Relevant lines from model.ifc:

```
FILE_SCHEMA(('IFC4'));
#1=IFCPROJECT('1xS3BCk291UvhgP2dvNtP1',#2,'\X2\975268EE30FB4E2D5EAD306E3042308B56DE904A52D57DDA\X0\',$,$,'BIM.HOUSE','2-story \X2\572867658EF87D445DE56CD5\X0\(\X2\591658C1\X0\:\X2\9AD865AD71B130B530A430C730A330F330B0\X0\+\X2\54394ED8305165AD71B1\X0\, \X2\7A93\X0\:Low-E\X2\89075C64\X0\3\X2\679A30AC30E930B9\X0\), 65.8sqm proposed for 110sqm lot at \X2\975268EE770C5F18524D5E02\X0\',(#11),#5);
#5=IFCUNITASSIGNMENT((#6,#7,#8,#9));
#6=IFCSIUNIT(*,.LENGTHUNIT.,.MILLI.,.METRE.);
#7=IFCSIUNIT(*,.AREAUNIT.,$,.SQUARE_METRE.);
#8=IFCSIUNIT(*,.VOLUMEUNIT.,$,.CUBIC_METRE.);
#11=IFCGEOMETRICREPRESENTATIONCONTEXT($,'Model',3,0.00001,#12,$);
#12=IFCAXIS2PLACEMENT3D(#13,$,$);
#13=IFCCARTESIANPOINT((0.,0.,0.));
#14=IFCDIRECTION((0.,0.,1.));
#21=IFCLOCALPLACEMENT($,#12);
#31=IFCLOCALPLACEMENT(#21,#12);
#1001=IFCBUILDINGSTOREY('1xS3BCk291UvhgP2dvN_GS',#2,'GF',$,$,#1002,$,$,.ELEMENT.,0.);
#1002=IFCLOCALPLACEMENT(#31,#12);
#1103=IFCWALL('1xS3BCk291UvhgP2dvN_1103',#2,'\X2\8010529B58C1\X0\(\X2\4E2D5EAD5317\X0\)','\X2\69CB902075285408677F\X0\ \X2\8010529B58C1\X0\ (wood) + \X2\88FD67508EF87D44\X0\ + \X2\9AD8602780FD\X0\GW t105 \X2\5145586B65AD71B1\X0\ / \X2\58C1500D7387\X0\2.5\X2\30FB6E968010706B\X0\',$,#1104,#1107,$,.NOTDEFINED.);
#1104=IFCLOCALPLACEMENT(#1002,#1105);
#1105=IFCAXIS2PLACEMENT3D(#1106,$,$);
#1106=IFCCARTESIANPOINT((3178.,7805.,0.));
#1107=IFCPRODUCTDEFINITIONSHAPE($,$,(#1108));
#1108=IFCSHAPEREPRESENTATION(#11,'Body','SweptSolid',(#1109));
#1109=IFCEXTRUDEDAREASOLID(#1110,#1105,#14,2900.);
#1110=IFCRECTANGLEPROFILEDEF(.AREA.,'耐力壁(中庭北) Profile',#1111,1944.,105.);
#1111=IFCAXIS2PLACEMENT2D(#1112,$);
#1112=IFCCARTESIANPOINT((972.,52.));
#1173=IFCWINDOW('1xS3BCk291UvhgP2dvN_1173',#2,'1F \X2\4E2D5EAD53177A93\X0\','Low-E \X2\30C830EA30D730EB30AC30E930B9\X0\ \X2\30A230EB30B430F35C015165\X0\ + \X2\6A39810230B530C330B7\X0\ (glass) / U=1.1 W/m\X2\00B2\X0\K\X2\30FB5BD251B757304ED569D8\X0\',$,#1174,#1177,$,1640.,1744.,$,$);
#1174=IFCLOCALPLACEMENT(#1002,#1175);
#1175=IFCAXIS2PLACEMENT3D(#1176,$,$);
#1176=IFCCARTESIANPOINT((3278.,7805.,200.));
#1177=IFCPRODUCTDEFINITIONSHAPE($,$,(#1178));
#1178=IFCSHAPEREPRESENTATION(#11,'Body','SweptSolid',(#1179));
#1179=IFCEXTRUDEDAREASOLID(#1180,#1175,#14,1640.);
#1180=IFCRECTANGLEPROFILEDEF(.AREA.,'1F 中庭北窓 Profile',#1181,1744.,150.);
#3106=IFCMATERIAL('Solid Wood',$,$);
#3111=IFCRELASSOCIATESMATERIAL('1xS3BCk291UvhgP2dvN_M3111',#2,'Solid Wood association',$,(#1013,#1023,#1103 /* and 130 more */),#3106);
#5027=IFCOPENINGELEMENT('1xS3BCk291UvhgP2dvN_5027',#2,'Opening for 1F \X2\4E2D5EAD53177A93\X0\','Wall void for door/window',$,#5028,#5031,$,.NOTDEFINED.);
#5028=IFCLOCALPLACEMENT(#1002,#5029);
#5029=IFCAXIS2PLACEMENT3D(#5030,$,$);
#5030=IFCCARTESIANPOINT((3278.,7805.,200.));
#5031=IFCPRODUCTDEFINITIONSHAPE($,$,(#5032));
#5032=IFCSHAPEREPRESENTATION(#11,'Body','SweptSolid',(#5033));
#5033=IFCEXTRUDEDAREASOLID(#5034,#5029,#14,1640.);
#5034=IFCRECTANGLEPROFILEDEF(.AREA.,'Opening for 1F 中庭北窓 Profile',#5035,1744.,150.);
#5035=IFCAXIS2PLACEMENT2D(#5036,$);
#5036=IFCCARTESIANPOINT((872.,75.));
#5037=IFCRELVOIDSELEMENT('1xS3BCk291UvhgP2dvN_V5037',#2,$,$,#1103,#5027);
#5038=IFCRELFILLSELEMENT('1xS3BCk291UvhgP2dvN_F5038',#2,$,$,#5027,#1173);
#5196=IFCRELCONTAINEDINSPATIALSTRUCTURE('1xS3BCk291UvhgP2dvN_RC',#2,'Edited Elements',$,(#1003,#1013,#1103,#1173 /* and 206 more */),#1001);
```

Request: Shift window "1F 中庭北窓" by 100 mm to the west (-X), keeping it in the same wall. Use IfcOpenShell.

```python
import ifcopenshell
import ifcopenshell.api.geometry
import ifcopenshell.util.placement

model = ifcopenshell.open("model.ifc")

window = model.by_guid("1xS3BCk291UvhgP2dvN_1173")
opening = window.FillsVoids[0].RelatingOpeningElement
wall = opening.VoidsElements[0].RelatingBuildingElement

wall_matrix = ifcopenshell.util.placement.get_local_placement(wall.ObjectPlacement)
shift = wall_matrix[:3, 0] * -100.0
before = ifcopenshell.util.placement.get_local_placement(window.ObjectPlacement)[:3, 3].copy()

# The window is not placed relative to its opening, so move both.
for product in (opening, window):
    matrix = ifcopenshell.util.placement.get_local_placement(product.ObjectPlacement)
    matrix[:3, 3] += shift
    ifcopenshell.api.geometry.edit_object_placement(model, product=product, matrix=matrix, is_si=False)

after = ifcopenshell.util.placement.get_local_placement(window.ObjectPlacement)[:3, 3]
print("window moved by", (after - before).round(3) + 0.0)

model.write("model_rev.ifc")
```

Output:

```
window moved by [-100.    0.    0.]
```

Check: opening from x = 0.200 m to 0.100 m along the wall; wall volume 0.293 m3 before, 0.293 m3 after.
